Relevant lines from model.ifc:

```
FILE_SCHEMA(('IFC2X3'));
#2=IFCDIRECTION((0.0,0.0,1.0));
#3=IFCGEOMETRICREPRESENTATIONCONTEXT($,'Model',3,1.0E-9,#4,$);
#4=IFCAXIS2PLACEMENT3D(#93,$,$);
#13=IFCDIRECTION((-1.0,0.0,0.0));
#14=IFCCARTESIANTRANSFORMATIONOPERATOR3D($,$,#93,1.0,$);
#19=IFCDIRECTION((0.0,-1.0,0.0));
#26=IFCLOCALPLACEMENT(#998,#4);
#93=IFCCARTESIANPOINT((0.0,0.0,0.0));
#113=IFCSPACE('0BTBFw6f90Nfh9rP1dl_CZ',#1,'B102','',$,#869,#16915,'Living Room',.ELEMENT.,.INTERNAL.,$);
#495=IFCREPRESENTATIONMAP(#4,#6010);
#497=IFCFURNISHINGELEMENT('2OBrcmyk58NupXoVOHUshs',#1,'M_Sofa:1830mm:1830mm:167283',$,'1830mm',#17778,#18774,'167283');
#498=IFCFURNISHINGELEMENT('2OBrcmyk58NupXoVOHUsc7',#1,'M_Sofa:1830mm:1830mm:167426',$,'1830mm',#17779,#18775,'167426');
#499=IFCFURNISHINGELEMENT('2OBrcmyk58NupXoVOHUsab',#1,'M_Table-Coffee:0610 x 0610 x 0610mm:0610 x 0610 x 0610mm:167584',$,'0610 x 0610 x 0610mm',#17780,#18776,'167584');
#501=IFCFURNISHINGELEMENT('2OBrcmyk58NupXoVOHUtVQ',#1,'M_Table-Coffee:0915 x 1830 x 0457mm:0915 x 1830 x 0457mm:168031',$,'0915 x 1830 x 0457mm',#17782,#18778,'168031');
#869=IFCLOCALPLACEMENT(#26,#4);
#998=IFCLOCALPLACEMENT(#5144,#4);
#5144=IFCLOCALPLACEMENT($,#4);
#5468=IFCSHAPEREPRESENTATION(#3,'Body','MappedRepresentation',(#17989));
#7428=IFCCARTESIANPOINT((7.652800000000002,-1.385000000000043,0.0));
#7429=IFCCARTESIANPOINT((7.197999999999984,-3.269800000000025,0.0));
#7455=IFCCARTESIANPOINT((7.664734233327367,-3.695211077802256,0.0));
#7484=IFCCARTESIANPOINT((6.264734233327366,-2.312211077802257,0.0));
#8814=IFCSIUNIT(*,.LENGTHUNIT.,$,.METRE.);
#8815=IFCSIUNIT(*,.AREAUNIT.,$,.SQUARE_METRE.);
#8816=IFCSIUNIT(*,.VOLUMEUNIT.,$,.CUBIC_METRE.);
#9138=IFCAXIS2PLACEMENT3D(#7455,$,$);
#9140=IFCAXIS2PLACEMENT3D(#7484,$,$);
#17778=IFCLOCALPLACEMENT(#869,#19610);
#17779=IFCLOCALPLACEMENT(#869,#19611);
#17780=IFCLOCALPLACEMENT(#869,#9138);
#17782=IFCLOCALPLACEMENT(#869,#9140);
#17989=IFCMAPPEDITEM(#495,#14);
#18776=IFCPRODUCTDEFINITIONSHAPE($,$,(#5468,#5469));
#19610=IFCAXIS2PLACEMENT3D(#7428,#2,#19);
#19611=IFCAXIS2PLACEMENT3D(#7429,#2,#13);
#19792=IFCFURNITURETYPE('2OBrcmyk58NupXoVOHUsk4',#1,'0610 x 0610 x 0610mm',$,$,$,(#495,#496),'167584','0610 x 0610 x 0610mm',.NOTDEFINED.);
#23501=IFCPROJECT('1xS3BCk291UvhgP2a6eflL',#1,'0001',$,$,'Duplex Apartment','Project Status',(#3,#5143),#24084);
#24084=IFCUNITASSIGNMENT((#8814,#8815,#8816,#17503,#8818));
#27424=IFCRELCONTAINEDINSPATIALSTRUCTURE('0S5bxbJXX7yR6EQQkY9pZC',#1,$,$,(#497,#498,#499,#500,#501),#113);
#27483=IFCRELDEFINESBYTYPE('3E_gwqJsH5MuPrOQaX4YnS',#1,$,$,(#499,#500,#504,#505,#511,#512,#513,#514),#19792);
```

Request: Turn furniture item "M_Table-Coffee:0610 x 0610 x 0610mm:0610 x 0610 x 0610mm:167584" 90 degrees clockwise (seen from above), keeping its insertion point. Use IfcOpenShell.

```python
import ifcopenshell
import ifcopenshell.api.geometry
import ifcopenshell.util.placement

model = ifcopenshell.open("model.ifc")

item = model.by_guid("2OBrcmyk58NupXoVOHUsab")
matrix = ifcopenshell.util.placement.get_local_placement(item.ObjectPlacement)
matrix = matrix @ ifcopenshell.util.placement.rotation(-90, "Z")
ifcopenshell.api.geometry.edit_object_placement(model, product=item, matrix=matrix, is_si=False)

print(ifcopenshell.util.placement.get_local_placement(item.ObjectPlacement).round(3) + 0.0)

model.write("model-out.ifc")
```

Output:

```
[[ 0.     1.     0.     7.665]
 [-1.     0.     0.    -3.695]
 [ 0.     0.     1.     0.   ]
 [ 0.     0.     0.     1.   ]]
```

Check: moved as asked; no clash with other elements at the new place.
